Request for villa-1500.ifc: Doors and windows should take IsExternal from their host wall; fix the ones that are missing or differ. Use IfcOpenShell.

First a look at what the model holds.

```python
import ifcopenshell
import ifcopenshell.util.element

model = ifcopenshell.open("villa-1500.ifc")
print(model.schema)
seen = {}
for e in model.by_type("IfcDoor") + model.by_type("IfcWindow"):
    if not e.FillsVoids:
        continue
    host = e.FillsVoids[0].RelatingOpeningElement.VoidsElements[0].RelatingBuildingElement
    own = ifcopenshell.util.element.get_pset(e, f"Pset_{e.is_a()[3:].removesuffix('StandardCase')}Common", "IsExternal")
    wall = ifcopenshell.util.element.get_pset(host, "Pset_WallCommon", "IsExternal")
    seen[e.is_a(), own, wall] = seen.get((e.is_a(), own, wall), 0) + 1
for (cls, own, wall), count in sorted(seen.items(), key=str):
    print(count, cls, "IsExternal:", own, "| host wall:", wall)
```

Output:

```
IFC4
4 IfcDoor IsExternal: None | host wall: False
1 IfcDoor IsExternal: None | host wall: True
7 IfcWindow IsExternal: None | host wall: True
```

```python
import ifcopenshell
import ifcopenshell.api.pset
import ifcopenshell.util.element

model = ifcopenshell.open("villa-1500.ifc")

count = 0
for ifc_class, pset_name in (("IfcDoor", "Pset_DoorCommon"), ("IfcWindow", "Pset_WindowCommon")):
    for e in model.by_type(ifc_class):
        if not e.FillsVoids:
            continue
        host = e.FillsVoids[0].RelatingOpeningElement.VoidsElements[0].RelatingBuildingElement
        external = ifcopenshell.util.element.get_pset(host, "Pset_WallCommon", "IsExternal")
        if external is None or ifcopenshell.util.element.get_pset(e, pset_name, "IsExternal") == external:
            continue
        pset = ifcopenshell.api.pset.add_pset(model, product=e, name=pset_name)
        ifcopenshell.api.pset.edit_pset(model, pset=pset, properties={"IsExternal": external})
        count += 1

print(count, "updated")

model.write("villa-1500-out.ifc")
```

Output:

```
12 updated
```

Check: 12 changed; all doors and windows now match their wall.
